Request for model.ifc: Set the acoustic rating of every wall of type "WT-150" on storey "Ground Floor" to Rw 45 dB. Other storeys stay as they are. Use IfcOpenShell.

First a look at what the model holds.

```python
import ifcopenshell
import ifcopenshell.util.element

model = ifcopenshell.open("model.ifc")
print(model.schema)
storey = next(s for s in model.by_type("IfcBuildingStorey") if s.Name == "Ground Floor")
walls = [e for e in ifcopenshell.util.element.get_decomposition(storey) if e.is_a("IfcWall")]
seen = {}
for e in walls:
    element_type = ifcopenshell.util.element.get_type(e)
    key = (element_type.Name if element_type != e and element_type else None, ifcopenshell.util.element.get_pset(e, "Pset_WallCommon", "AcousticRating"))
    seen[key] = seen.get(key, 0) + 1
for (name, value), count in sorted(seen.items(), key=str):
    print(count, "x", name, "|", value)
```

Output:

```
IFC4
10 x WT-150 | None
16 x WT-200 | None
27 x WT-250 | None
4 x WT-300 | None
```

```python
import ifcopenshell
import ifcopenshell.api.pset
import ifcopenshell.util.element

model = ifcopenshell.open("model.ifc")

storey = next(s for s in model.by_type("IfcBuildingStorey") if s.Name == "Ground Floor")
walls = [e for e in ifcopenshell.util.element.get_decomposition(storey) if e.is_a("IfcWall")]

count = 0
for e in walls:
    element_type = ifcopenshell.util.element.get_type(e)
    if element_type in (None, e) or element_type.Name != "WT-150":
        continue
    # add_pset returns the element's existing set when there is one.
    pset = ifcopenshell.api.pset.add_pset(model, product=e, name="Pset_WallCommon")
    ifcopenshell.api.pset.edit_pset(model, pset=pset, properties={"AcousticRating": "Rw 45 dB"})
    count += 1

print(count, "walls updated")

model.write("model_v2.ifc")
```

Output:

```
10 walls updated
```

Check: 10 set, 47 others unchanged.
